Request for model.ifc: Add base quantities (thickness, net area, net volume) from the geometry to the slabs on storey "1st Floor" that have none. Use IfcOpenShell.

First a look at what the model holds.

```python
import ifcopenshell
import ifcopenshell.util.element
import ifcopenshell.util.unit

model = ifcopenshell.open("model.ifc")
print(model.schema)
for unit_type in ("LENGTHUNIT", "AREAUNIT", "VOLUMEUNIT"):
    print(unit_type, ifcopenshell.util.unit.calculate_unit_scale(model, unit_type))
storey = next(s for s in model.by_type("IfcBuildingStorey") if s.Name == "1st Floor")
slabs = [e for e in ifcopenshell.util.element.get_decomposition(storey) if e.is_a("IfcSlab")]
for e in sorted(slabs, key=lambda e: e.id()):
    print(e.id(), e.is_a(), e.Name, list(ifcopenshell.util.element.get_psets(e, qtos_only=True)), sep=" | ")
```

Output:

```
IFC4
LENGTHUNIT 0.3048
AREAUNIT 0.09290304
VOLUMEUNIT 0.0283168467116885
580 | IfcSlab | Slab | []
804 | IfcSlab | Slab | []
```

```python
import ifcopenshell
import ifcopenshell.api.pset
import ifcopenshell.geom
import ifcopenshell.util.element
import ifcopenshell.util.shape
import ifcopenshell.util.unit

model = ifcopenshell.open("model.ifc")
unit_scale = ifcopenshell.util.unit.calculate_unit_scale(model)
area_scale = ifcopenshell.util.unit.calculate_unit_scale(model, "AREAUNIT")
volume_scale = ifcopenshell.util.unit.calculate_unit_scale(model, "VOLUMEUNIT")
settings = ifcopenshell.geom.settings()

storey = next(s for s in model.by_type("IfcBuildingStorey") if s.Name == "1st Floor")
slabs = [e for e in ifcopenshell.util.element.get_decomposition(storey) if e.is_a("IfcSlab")]

for e in sorted(slabs, key=lambda e: e.id()):
    if ifcopenshell.util.element.get_psets(e, qtos_only=True, should_inherit=False):
        continue
    # Geometry comes back in metres, in the element's own axes.
    shape = ifcopenshell.geom.create_shape(settings, e)
    values = {
        "Width": ifcopenshell.util.shape.get_z(shape.geometry) / unit_scale,
        "NetArea": ifcopenshell.util.shape.get_footprint_area(shape.geometry) / area_scale,
        "NetVolume": ifcopenshell.util.shape.get_volume(shape.geometry) / volume_scale,
    }
    qto = ifcopenshell.api.pset.add_qto(model, product=e, name="Qto_SlabBaseQuantities")
    ifcopenshell.api.pset.edit_qto(model, qto=qto, properties=values)
    print(e.id(), {k: round(v, 3) for k, v in values.items()})

model.write("model_edited.ifc")
```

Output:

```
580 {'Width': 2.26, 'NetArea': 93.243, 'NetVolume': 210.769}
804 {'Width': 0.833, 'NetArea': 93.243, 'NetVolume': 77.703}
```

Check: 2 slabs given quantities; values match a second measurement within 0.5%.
